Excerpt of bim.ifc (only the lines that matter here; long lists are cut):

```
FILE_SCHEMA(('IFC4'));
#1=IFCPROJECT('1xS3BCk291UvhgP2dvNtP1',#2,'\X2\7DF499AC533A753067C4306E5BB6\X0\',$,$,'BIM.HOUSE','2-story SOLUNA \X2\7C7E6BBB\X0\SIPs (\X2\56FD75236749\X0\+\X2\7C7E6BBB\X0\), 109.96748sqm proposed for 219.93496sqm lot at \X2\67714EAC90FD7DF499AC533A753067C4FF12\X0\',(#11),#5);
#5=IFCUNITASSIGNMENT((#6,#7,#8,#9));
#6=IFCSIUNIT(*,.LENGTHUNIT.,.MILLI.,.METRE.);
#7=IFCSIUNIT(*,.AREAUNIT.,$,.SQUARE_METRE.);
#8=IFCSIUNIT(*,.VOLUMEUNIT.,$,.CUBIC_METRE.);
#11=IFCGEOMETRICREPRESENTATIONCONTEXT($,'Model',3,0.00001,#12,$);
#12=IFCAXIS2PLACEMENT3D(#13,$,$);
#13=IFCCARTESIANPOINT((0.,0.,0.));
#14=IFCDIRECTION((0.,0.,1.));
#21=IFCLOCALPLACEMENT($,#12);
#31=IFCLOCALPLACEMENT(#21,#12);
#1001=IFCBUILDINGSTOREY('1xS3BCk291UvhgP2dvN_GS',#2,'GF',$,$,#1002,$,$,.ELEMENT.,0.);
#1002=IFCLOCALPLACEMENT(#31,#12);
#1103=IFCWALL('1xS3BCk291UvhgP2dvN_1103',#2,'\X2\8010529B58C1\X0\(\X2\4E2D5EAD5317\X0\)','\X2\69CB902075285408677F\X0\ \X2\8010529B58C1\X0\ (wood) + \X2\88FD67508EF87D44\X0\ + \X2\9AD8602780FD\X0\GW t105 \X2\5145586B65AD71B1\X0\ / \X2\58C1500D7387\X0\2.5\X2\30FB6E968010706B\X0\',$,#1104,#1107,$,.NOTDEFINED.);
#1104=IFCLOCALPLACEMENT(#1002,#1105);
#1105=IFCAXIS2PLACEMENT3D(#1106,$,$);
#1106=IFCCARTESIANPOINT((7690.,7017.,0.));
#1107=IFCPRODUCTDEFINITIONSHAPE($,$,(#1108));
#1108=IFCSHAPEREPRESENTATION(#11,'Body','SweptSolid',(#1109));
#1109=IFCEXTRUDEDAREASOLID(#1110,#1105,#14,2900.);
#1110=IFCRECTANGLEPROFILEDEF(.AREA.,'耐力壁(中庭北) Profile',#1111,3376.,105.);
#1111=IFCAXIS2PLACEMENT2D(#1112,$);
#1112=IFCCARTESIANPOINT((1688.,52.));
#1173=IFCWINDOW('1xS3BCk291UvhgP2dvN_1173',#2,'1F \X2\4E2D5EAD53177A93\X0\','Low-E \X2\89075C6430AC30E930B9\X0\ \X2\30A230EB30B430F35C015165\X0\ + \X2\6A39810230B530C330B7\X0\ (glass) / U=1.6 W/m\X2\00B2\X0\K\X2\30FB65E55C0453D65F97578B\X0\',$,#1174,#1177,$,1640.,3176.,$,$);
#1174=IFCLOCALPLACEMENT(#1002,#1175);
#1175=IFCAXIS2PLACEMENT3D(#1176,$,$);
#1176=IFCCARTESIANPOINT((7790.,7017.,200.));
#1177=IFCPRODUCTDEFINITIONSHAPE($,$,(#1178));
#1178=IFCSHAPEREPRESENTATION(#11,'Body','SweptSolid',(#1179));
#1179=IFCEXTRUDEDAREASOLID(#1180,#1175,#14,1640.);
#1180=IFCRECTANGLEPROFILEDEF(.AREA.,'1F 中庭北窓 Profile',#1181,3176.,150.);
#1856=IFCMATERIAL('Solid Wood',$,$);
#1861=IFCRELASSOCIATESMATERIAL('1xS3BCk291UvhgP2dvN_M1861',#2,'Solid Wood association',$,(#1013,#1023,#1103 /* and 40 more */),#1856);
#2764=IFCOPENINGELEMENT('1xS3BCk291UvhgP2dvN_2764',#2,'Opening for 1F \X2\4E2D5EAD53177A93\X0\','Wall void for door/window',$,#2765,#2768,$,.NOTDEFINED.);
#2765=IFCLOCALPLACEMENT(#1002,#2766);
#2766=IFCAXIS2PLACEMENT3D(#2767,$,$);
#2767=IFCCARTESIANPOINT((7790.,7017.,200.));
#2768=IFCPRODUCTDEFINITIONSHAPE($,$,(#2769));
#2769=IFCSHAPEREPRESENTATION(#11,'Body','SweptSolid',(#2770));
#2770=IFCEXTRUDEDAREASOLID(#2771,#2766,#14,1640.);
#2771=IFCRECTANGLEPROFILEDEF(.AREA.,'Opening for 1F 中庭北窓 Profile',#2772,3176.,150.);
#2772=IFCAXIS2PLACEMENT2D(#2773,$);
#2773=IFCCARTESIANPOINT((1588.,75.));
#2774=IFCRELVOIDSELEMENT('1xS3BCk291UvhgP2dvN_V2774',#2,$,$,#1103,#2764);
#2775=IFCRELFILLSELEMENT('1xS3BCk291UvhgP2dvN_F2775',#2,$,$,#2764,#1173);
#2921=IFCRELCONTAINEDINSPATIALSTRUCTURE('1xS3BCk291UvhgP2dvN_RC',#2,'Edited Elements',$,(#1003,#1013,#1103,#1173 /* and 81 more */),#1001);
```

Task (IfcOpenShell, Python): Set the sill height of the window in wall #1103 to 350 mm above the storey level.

```python
import numpy as np
import ifcopenshell
import ifcopenshell.api.geometry
import ifcopenshell.geom
import ifcopenshell.util.element
import ifcopenshell.util.placement
import ifcopenshell.util.shape
import ifcopenshell.util.unit

model = ifcopenshell.open("bim.ifc")
unit_scale = ifcopenshell.util.unit.calculate_unit_scale(model)

window = model.by_id(1173)
opening = window.FillsVoids[0].RelatingOpeningElement
storey = ifcopenshell.util.element.get_container(window, ifc_class="IfcBuildingStorey")
level = ifcopenshell.util.placement.get_local_placement(storey.ObjectPlacement)[2, 3]

# The opening's origin need not be at the sill, so measure its lowest point.
shape = ifcopenshell.geom.create_shape(ifcopenshell.geom.settings(), opening)
bottom = ifcopenshell.util.shape.get_shape_bottom_elevation(shape, shape.geometry) / unit_scale
dz = level + 0.35 / unit_scale - bottom

shift = np.array([0.0, 0.0, dz])
# The window is not placed relative to its opening, so move both.
for product in (opening, window):
    matrix = ifcopenshell.util.placement.get_local_placement(product.ObjectPlacement)
    matrix[:3, 3] += shift
    ifcopenshell.api.geometry.edit_object_placement(model, product=product, matrix=matrix, is_si=False)

print(f"moved by {dz * unit_scale:+.3f} m")

model.write("bim_v2.ifc")
```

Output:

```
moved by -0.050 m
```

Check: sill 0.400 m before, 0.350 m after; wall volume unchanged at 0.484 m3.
